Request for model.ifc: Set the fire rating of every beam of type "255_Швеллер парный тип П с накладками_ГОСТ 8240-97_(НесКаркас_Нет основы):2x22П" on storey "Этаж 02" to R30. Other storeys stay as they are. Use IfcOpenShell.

First a look at what the model holds.

```python
import ifcopenshell
import ifcopenshell.util.element

model = ifcopenshell.open("model.ifc")
print(model.schema)
storey = next(s for s in model.by_type("IfcBuildingStorey") if s.Name == "Этаж 02")
beams = [e for e in ifcopenshell.util.element.get_decomposition(storey) if e.is_a("IfcBeam")]
seen = {}
for e in beams:
    element_type = ifcopenshell.util.element.get_type(e)
    key = (element_type.Name if element_type != e and element_type else None, ifcopenshell.util.element.get_pset(e, "Pset_BeamCommon", "FireRating"))
    seen[key] = seen.get(key, 0) + 1
for (name, value), count in sorted(seen.items(), key=str):
    print(count, "x", name, "|", value)
```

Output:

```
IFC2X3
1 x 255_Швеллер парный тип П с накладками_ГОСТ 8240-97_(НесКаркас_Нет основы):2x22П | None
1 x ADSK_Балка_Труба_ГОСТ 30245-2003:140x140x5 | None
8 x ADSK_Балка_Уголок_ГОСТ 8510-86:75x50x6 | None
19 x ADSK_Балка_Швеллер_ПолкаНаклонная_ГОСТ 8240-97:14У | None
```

```python
import ifcopenshell
import ifcopenshell.api.pset
import ifcopenshell.util.element

model = ifcopenshell.open("model.ifc")

storey = next(s for s in model.by_type("IfcBuildingStorey") if s.Name == "Этаж 02")
beams = [e for e in ifcopenshell.util.element.get_decomposition(storey) if e.is_a("IfcBeam")]

count = 0
for e in beams:
    element_type = ifcopenshell.util.element.get_type(e)
    if element_type in (None, e) or element_type.Name != "255_Швеллер парный тип П с накладками_ГОСТ 8240-97_(НесКаркас_Нет основы):2x22П":
        continue
    # add_pset returns the element's existing set when there is one.
    pset = ifcopenshell.api.pset.add_pset(model, product=e, name="Pset_BeamCommon")
    ifcopenshell.api.pset.edit_pset(model, pset=pset, properties={"FireRating": "R30"})
    count += 1

print(count, "beams updated")

model.write("model-out.ifc")
```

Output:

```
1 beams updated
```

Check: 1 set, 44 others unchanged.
